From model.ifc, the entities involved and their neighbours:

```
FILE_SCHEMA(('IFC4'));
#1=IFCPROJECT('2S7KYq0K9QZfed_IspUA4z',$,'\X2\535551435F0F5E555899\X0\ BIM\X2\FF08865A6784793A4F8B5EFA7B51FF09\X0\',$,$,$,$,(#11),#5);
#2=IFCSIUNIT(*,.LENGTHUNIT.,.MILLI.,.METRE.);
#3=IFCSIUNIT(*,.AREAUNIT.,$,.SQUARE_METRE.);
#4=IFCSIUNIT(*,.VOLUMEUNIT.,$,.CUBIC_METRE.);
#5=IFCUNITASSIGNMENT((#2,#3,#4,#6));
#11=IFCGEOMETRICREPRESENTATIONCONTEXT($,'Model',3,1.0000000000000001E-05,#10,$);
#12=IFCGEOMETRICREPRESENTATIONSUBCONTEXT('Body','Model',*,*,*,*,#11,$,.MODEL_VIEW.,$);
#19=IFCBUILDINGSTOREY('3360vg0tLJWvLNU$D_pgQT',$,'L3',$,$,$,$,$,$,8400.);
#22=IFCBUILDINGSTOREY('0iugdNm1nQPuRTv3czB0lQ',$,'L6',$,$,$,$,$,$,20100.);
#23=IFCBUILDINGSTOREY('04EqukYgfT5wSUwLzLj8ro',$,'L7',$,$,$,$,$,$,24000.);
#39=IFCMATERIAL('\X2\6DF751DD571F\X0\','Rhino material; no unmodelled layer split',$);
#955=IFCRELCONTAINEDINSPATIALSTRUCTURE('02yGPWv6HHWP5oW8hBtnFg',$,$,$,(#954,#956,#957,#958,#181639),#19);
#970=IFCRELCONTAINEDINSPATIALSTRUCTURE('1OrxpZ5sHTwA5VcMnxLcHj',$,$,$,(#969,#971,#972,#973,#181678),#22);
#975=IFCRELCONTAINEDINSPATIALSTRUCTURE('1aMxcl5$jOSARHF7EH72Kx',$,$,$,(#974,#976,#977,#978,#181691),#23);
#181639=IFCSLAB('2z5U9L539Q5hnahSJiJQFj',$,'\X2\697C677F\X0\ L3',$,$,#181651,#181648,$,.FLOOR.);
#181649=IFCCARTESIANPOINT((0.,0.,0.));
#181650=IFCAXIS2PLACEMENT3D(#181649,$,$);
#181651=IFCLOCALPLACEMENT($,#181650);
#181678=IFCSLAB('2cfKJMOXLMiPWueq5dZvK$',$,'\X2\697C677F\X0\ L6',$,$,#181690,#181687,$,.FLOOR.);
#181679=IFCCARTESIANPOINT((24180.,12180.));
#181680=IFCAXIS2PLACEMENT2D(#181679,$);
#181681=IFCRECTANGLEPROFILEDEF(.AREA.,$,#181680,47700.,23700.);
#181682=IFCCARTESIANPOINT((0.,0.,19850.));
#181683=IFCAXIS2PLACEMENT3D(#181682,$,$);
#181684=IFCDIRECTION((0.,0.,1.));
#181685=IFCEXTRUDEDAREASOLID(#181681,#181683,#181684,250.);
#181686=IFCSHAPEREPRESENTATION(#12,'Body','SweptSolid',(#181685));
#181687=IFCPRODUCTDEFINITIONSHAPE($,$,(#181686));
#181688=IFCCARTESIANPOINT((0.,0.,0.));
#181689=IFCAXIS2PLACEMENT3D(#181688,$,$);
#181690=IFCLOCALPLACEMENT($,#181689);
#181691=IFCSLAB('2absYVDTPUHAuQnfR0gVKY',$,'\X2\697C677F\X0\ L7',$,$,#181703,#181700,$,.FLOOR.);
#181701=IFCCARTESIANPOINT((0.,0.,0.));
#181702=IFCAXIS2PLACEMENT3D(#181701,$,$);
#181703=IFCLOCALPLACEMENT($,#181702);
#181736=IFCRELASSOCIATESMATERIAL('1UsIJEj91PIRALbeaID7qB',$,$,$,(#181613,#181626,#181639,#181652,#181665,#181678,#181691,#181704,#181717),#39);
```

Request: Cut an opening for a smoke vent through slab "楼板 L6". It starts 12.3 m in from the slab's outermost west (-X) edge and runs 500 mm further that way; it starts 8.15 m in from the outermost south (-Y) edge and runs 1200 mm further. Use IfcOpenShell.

```python
import numpy as np
import ifcopenshell
import ifcopenshell.api.feature
import ifcopenshell.api.geometry
import ifcopenshell.api.root
import ifcopenshell.geom
import ifcopenshell.util.placement
import ifcopenshell.util.representation
import ifcopenshell.util.shape
import ifcopenshell.util.unit

model = ifcopenshell.open("model.ifc")
unit_scale = ifcopenshell.util.unit.calculate_unit_scale(model)
settings = ifcopenshell.geom.settings()


def volume(element):
    """Net volume in cubic metres, openings subtracted."""
    shape = ifcopenshell.geom.create_shape(settings, element)
    return ifcopenshell.util.shape.get_volume(shape.geometry)


slab = model.by_guid("2cfKJMOXLMiPWueq5dZvK$")
before = volume(slab)

# Extent in the slab's own axes, in metres. The edges named are its -X and -Y sides.
slab_shape = ifcopenshell.geom.create_shape(settings, slab)
vertices = ifcopenshell.util.shape.get_vertices(slab_shape.geometry)
x_min, y_min, bottom = vertices.min(axis=0)
top = vertices[:, 2].max()

opening = ifcopenshell.api.root.create_entity(model, ifc_class="IfcOpeningElement", name="Smoke vent opening", predefined_type="OPENING")
context = ifcopenshell.util.representation.get_context(model, "Model", "Body", "MODEL_VIEW")
width, depth = 0.5, 1.2
outline = [(0.0, 0.0), (width, 0.0), (width, depth), (0.0, depth), (0.0, 0.0)]
# Overshoot both faces by 50 mm so the cut is clean.
shape = ifcopenshell.api.geometry.add_slab_representation(
    model, context=context, depth=top - bottom + 0.1, polyline=outline
)
ifcopenshell.api.geometry.assign_representation(model, product=opening, representation=shape)

matrix = ifcopenshell.util.placement.get_local_placement(slab.ObjectPlacement)
matrix[:, 3] = matrix @ np.append(np.array([x_min + 12.3, y_min + 8.15, bottom - 0.05]) / unit_scale, 1.0)
ifcopenshell.api.geometry.edit_object_placement(model, product=opening, matrix=matrix, is_si=False)
ifcopenshell.api.feature.add_feature(model, feature=opening, element=slab)

after = volume(slab)

print(f"slab volume {before:.3f} -> {after:.3f} m3")

model.write("model_v2.ifc")
```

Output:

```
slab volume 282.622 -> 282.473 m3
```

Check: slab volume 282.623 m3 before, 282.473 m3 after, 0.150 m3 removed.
